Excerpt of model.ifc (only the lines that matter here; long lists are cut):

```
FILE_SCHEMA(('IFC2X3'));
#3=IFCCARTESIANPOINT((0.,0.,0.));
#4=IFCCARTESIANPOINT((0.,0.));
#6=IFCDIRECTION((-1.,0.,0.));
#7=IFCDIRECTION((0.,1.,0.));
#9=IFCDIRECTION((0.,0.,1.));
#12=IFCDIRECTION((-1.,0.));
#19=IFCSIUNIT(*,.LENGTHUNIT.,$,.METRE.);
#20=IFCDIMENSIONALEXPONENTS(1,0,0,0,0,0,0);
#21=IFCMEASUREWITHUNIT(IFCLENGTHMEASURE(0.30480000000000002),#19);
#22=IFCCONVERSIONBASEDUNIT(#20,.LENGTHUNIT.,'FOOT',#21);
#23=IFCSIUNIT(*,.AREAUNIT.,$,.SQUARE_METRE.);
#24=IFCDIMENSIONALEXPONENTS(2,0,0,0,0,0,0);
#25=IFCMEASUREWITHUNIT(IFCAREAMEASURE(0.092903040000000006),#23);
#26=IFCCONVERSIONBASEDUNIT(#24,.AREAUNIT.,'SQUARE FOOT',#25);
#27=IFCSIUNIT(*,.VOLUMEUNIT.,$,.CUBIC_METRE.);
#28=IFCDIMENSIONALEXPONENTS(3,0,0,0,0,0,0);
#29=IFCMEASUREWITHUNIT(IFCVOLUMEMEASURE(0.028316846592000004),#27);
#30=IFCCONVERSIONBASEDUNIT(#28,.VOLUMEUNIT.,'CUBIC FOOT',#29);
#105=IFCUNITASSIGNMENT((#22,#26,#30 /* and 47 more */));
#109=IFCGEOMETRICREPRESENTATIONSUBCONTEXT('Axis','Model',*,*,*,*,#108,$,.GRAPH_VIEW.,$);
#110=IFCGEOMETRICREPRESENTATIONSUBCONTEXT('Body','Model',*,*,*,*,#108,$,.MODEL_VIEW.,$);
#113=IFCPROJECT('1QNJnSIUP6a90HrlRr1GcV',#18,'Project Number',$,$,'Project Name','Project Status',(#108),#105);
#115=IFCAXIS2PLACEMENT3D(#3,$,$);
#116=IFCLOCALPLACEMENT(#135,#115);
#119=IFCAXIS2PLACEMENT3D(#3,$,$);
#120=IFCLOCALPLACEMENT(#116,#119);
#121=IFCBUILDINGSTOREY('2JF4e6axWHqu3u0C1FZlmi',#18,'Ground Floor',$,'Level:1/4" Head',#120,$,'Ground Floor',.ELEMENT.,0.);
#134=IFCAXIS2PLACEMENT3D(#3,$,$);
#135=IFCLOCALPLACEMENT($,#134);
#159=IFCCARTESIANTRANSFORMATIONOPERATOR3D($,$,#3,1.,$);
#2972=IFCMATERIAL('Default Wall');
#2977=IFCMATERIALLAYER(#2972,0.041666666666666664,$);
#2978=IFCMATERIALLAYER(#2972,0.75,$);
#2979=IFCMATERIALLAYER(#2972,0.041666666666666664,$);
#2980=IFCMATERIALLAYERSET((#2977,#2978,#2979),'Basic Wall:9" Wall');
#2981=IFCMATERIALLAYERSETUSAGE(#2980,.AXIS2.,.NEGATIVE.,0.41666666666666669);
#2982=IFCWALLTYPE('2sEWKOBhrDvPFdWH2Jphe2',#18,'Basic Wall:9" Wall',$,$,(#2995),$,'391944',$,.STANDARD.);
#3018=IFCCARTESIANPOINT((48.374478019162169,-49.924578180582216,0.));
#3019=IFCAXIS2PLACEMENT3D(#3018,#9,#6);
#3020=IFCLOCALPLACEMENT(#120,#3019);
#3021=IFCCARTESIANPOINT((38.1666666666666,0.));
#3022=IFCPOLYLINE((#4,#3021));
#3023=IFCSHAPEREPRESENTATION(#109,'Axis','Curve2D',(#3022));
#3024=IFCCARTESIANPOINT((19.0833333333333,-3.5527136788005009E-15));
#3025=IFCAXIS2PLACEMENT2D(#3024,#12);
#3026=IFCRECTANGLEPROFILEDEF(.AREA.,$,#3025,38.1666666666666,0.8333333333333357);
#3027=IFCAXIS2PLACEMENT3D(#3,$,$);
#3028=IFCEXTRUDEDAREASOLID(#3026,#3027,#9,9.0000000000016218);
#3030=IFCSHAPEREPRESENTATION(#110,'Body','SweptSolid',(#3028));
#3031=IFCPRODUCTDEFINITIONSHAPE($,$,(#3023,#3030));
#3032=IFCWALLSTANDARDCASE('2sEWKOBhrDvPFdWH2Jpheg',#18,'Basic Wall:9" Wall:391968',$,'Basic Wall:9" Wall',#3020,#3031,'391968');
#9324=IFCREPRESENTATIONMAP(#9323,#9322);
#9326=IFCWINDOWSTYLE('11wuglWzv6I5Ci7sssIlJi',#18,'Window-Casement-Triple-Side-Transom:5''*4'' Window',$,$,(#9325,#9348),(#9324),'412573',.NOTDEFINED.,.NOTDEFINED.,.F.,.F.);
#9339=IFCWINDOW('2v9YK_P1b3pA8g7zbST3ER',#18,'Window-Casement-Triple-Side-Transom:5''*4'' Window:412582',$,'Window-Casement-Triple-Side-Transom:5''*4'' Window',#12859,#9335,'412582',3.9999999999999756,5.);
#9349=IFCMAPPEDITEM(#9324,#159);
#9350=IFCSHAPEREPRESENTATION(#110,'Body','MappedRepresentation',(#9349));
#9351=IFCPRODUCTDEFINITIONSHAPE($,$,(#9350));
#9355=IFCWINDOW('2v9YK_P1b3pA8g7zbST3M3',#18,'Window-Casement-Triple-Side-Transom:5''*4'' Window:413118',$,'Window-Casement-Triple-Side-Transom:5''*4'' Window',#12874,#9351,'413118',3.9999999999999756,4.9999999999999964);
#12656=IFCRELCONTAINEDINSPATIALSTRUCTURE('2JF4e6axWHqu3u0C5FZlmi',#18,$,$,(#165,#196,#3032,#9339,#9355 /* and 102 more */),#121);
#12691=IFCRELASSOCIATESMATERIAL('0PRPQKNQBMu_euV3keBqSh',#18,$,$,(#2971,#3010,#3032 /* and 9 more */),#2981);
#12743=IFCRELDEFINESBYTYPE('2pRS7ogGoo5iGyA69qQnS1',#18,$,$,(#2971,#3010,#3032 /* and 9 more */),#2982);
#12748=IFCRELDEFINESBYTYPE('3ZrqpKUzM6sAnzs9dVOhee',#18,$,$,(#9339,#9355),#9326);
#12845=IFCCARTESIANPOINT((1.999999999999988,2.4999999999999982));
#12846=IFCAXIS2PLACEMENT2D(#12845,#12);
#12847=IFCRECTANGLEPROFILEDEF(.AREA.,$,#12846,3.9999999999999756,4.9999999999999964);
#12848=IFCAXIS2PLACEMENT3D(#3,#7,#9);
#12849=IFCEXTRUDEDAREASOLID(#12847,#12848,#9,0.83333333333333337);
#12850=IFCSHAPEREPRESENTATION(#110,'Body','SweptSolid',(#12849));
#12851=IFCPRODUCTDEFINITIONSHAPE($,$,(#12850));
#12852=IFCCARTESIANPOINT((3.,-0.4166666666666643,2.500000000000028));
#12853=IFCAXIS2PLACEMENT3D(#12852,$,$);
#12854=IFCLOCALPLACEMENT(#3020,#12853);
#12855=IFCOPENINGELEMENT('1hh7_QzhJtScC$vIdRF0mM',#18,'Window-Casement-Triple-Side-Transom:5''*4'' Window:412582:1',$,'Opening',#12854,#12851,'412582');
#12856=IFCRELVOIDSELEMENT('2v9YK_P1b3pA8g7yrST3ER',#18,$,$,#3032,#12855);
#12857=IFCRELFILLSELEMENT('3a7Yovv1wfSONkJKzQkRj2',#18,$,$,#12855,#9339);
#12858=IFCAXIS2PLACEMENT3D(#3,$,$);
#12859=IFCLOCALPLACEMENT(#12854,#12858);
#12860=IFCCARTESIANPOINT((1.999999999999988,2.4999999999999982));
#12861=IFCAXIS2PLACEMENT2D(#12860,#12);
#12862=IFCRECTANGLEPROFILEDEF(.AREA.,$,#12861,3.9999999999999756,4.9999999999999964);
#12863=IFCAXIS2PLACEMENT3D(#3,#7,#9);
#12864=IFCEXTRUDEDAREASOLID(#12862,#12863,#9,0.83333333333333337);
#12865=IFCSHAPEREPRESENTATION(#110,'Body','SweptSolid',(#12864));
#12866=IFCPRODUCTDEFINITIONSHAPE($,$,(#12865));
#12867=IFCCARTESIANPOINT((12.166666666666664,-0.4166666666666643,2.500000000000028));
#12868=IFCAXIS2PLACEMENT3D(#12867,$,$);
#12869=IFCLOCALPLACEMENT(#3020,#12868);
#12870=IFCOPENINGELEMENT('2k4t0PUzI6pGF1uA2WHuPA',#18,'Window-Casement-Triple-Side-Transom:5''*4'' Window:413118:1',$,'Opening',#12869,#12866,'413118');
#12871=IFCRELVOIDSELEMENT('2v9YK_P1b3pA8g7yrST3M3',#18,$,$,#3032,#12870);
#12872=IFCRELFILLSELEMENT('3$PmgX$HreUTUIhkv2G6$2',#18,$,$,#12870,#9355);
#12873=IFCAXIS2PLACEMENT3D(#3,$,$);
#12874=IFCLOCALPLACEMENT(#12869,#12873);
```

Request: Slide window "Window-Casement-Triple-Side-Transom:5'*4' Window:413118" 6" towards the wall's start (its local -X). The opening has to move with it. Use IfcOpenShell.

```python
import ifcopenshell
import ifcopenshell.api.geometry
import ifcopenshell.util.placement
import ifcopenshell.util.unit

model = ifcopenshell.open("model.ifc")
unit_scale = ifcopenshell.util.unit.calculate_unit_scale(model)

window = model.by_id(9355)
opening = window.FillsVoids[0].RelatingOpeningElement
wall = opening.VoidsElements[0].RelatingBuildingElement

wall_matrix = ifcopenshell.util.placement.get_local_placement(wall.ObjectPlacement)
shift = wall_matrix[:3, 0] * -6 * 0.0254 / unit_scale
before = ifcopenshell.util.placement.get_local_placement(window.ObjectPlacement)[:3, 3].copy()

# The window is placed relative to its opening, so it follows when the opening moves.
matrix = ifcopenshell.util.placement.get_local_placement(opening.ObjectPlacement)
matrix[:3, 3] += shift
ifcopenshell.api.geometry.edit_object_placement(
    model, product=opening, matrix=matrix, is_si=False, should_transform_children=True
)

after = ifcopenshell.util.placement.get_local_placement(window.ObjectPlacement)[:3, 3]
print("window moved by", (after - before).round(3) + 0.0)

model.write("model_v2.ifc")
```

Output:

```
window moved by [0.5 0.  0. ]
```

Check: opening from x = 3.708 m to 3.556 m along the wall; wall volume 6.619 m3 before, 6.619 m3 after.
